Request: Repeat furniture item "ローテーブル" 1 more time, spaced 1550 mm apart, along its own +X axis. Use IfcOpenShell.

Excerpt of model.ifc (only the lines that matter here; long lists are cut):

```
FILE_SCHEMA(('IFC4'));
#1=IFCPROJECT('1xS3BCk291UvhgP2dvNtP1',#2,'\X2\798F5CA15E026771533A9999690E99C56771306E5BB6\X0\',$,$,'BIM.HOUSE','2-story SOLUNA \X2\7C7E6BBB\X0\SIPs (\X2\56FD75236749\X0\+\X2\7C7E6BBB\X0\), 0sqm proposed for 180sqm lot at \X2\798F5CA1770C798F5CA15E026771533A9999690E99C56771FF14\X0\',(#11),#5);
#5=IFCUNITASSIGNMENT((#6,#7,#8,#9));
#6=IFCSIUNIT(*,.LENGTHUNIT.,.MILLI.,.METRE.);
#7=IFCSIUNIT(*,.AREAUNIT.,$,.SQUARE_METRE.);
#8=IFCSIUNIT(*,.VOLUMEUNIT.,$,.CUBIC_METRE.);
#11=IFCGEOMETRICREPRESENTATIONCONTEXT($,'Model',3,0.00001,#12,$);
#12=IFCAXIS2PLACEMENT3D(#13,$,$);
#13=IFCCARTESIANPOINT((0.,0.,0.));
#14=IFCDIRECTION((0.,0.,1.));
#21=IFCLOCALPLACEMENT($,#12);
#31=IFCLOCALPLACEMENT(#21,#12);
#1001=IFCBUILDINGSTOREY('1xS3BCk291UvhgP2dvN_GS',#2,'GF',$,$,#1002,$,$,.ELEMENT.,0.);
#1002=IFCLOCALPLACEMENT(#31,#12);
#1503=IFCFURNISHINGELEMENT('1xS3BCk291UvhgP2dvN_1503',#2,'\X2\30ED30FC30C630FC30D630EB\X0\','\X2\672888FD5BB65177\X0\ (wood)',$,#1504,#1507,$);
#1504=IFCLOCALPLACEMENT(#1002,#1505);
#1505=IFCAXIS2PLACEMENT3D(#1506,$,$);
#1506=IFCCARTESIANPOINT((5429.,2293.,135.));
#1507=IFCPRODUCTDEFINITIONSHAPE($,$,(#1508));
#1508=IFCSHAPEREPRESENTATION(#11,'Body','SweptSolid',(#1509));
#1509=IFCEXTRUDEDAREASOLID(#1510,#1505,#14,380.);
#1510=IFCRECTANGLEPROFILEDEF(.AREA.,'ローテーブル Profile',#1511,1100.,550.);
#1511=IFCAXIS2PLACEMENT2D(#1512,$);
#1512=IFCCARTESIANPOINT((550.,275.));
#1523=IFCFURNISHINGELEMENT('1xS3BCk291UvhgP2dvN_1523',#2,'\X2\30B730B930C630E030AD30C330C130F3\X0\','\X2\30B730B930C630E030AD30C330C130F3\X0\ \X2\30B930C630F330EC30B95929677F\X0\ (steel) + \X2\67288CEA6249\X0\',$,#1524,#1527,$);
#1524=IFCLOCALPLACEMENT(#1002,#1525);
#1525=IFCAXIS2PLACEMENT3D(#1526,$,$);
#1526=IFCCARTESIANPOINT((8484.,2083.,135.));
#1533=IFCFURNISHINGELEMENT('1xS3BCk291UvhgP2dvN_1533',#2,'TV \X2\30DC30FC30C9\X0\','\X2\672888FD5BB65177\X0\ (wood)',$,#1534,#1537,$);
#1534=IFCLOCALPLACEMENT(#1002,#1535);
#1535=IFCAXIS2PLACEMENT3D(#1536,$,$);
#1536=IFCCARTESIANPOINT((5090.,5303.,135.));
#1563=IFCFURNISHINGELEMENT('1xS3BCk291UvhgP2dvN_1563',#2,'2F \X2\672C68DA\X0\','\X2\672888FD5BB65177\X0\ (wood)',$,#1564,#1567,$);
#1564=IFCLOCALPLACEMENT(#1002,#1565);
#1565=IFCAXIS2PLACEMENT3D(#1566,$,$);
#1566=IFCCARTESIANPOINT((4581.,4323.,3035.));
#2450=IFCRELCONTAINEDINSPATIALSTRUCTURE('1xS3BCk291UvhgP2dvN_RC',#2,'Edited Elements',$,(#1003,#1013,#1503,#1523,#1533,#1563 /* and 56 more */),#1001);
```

```python
import ifcopenshell
import ifcopenshell.api.geometry
import ifcopenshell.api.root
import ifcopenshell.util.element
import ifcopenshell.util.placement

model = ifcopenshell.open("model.ifc")


def reuse_history(source, copy):
    """copy_class also copies each property set's owner history, people and application; keep the originals."""
    for rel in copy.IsDefinedBy:
        if rel.is_a("IfcRelDefinesByProperties") and (history := rel.RelatingPropertyDefinition.OwnerHistory):
            rel.RelatingPropertyDefinition.OwnerHistory = source.OwnerHistory
            ifcopenshell.util.element.remove_deep2(model, history)


source = model.by_guid("1xS3BCk291UvhgP2dvN_1503")
base = ifcopenshell.util.placement.get_local_placement(source.ObjectPlacement)
step = base[:3, 0] * 1550.0

for i in range(1, 2):
    copy = ifcopenshell.api.root.copy_class(model, product=source)
    copy.Representation = ifcopenshell.util.element.copy_deep(
        model, source.Representation, exclude=["IfcGeometricRepresentationContext", "IfcRepresentationMap"]
    )
    reuse_history(source, copy)
    matrix = base.copy()
    matrix[:3, 3] += i * step
    print("added at", matrix[:3, 3].round(3) + 0.0)
    ifcopenshell.api.geometry.edit_object_placement(model, product=copy, matrix=matrix, is_si=False)

model.write("model-out.ifc")
```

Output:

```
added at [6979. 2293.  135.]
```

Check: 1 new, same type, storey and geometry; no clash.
